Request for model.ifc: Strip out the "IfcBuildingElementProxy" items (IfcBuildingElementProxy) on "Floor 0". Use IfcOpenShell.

First a look at what the model holds.

```python
import ifcopenshell
import ifcopenshell.util.element

model = ifcopenshell.open("model.ifc")
print(model.schema)
storey = next(s for s in model.by_type("IfcBuildingStorey") if s.Name == "Floor 0")
proxies = [e for e in ifcopenshell.util.element.get_decomposition(storey) if e.is_a("IfcBuildingElementProxy")]
seen = {}
for e in proxies:
    element_type = ifcopenshell.util.element.get_type(e)
    name = element_type.Name if element_type not in (None, e) else None
    seen[name] = seen.get(name, 0) + 1
for name, count in sorted(seen.items(), key=str):
    print(count, "x", name)
```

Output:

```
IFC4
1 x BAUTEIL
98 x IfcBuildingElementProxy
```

```python
import ifcopenshell
import ifcopenshell.api.root
import ifcopenshell.util.element

model = ifcopenshell.open("model.ifc")

storey = next(s for s in model.by_type("IfcBuildingStorey") if s.Name == "Floor 0")
proxies = [e for e in ifcopenshell.util.element.get_decomposition(storey) if e.is_a("IfcBuildingElementProxy")]
targets = [e for e in proxies if (t := ifcopenshell.util.element.get_type(e)) not in (None, e) and t.Name == "IfcBuildingElementProxy"]

for e in targets:
    ifcopenshell.api.root.remove_product(model, product=e)
print(len(targets), "removed")

model.write("model_v2.ifc")
```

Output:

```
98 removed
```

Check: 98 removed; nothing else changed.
